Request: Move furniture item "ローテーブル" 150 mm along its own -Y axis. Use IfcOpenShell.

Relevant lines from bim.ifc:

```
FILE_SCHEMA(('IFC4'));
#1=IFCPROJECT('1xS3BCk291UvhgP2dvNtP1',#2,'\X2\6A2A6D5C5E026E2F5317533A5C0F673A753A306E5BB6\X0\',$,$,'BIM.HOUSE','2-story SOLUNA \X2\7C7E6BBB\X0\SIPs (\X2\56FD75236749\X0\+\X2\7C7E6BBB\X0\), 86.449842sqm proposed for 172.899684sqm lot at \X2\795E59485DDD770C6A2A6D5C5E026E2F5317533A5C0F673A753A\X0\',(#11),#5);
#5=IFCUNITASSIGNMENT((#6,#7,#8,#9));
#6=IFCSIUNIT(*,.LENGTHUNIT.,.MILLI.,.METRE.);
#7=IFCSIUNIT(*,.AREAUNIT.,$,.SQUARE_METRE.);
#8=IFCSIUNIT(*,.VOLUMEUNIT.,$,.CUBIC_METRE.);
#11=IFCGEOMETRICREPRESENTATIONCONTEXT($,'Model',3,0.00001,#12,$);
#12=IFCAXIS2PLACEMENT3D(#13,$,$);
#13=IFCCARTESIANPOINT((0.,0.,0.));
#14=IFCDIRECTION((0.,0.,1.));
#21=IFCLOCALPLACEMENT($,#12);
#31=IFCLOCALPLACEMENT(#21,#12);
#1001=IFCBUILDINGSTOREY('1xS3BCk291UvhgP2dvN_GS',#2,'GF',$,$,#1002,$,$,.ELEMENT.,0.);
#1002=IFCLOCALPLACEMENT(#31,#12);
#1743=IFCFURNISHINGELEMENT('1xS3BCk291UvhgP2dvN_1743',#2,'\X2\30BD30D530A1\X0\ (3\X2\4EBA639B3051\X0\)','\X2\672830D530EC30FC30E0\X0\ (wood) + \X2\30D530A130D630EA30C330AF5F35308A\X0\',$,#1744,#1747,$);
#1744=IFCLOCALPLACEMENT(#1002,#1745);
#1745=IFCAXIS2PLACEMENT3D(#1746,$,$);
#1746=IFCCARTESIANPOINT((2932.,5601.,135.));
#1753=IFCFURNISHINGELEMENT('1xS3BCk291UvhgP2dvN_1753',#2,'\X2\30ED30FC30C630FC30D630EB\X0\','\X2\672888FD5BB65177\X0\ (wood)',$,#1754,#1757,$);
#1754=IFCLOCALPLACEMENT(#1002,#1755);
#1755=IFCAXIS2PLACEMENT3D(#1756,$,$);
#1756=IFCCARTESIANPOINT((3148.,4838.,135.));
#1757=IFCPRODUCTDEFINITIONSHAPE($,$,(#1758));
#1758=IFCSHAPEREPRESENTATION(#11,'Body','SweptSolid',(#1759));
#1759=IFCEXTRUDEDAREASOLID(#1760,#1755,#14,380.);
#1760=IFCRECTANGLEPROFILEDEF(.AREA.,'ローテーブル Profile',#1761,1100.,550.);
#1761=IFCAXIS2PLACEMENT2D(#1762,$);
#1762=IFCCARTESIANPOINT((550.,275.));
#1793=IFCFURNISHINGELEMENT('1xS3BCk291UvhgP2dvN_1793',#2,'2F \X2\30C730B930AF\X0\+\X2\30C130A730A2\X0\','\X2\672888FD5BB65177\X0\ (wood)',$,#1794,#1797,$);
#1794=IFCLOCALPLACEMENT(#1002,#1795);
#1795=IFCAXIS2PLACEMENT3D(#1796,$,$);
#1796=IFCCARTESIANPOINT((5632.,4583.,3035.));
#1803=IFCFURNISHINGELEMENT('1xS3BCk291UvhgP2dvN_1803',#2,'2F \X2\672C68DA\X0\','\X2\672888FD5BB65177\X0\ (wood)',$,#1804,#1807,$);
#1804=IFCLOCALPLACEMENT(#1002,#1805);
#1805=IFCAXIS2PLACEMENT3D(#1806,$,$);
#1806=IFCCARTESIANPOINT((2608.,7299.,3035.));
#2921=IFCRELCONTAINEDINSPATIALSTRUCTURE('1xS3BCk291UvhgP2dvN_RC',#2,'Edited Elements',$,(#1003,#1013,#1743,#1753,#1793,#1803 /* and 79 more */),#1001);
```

```python
import ifcopenshell
import ifcopenshell.api.geometry
import ifcopenshell.util.placement

model = ifcopenshell.open("bim.ifc")

item = model.by_guid("1xS3BCk291UvhgP2dvN_1753")
matrix = ifcopenshell.util.placement.get_local_placement(item.ObjectPlacement)
matrix[:3, 3] -= matrix[:3, 1] * 150.0
ifcopenshell.api.geometry.edit_object_placement(model, product=item, matrix=matrix, is_si=False)

print(ifcopenshell.util.placement.get_local_placement(item.ObjectPlacement).round(3) + 0.0)

model.write("bim_updated.ifc")
```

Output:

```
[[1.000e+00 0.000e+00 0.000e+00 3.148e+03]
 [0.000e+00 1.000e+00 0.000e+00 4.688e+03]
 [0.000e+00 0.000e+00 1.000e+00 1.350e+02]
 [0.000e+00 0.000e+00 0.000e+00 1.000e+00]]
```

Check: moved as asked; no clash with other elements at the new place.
